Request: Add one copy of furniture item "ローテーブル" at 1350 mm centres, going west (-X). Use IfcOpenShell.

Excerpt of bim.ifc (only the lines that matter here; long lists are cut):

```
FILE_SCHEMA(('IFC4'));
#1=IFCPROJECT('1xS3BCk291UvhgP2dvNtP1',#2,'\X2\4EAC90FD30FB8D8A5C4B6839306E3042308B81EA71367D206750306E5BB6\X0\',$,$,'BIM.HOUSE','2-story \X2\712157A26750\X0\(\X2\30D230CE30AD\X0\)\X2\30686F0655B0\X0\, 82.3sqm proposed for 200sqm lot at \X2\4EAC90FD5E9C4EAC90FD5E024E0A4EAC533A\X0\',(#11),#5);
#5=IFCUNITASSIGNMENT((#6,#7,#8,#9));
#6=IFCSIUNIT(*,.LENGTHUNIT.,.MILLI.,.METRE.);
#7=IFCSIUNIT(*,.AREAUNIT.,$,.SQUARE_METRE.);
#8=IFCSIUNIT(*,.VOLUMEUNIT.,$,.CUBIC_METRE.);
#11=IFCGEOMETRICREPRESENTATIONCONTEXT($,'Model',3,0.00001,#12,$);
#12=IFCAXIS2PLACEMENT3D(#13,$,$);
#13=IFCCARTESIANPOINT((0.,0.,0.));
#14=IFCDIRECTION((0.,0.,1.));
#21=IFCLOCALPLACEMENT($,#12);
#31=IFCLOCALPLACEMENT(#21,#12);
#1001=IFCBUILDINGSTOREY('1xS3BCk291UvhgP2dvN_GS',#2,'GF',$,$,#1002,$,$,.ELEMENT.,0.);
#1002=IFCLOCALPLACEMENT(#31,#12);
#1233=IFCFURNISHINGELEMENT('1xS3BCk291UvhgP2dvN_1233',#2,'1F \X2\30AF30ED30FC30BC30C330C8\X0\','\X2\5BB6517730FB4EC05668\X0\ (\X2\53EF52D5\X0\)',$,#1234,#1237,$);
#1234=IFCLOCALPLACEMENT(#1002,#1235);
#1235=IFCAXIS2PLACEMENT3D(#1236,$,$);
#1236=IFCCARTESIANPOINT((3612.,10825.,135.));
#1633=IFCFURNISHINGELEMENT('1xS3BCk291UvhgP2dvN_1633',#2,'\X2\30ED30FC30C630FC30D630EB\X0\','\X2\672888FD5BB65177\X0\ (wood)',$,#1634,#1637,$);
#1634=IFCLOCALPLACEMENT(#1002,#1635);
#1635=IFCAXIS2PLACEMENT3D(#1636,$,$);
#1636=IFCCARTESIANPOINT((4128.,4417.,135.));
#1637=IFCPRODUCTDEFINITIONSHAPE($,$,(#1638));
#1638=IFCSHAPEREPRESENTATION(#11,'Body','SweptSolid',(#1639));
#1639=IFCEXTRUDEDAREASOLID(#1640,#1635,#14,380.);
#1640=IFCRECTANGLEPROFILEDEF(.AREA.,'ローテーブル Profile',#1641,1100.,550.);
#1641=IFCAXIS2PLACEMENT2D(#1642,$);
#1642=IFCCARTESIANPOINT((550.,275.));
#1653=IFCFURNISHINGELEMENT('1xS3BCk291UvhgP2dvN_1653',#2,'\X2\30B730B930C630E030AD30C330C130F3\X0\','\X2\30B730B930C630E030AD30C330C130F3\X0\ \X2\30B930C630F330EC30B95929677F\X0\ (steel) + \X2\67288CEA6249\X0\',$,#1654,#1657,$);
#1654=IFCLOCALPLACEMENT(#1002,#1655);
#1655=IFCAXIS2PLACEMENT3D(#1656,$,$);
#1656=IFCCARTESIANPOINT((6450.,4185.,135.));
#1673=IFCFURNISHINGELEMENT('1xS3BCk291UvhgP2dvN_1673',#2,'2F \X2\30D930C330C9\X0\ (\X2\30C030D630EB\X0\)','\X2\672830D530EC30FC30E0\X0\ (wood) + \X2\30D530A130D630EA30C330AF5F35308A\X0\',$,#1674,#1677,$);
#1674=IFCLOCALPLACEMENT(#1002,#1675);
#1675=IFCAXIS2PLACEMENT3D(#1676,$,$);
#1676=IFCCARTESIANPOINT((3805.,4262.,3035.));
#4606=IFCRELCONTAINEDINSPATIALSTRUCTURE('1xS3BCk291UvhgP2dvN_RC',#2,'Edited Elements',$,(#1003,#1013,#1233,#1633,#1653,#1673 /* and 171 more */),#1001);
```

```python
import numpy as np
import ifcopenshell
import ifcopenshell.api.geometry
import ifcopenshell.api.root
import ifcopenshell.util.element
import ifcopenshell.util.placement
import ifcopenshell.util.unit

model = ifcopenshell.open("bim.ifc")
unit_scale = ifcopenshell.util.unit.calculate_unit_scale(model)


def reuse_history(source, copy):
    """copy_class also copies each property set's owner history, people and application; keep the originals."""
    for rel in copy.IsDefinedBy:
        if rel.is_a("IfcRelDefinesByProperties") and (history := rel.RelatingPropertyDefinition.OwnerHistory):
            rel.RelatingPropertyDefinition.OwnerHistory = source.OwnerHistory
            ifcopenshell.util.element.remove_deep2(model, history)


source = model.by_guid("1xS3BCk291UvhgP2dvN_1633")
base = ifcopenshell.util.placement.get_local_placement(source.ObjectPlacement)
step = np.array([-1.0, 0.0, 0.0]) * 1.35 / unit_scale

for i in range(1, 2):
    copy = ifcopenshell.api.root.copy_class(model, product=source)
    copy.Representation = ifcopenshell.util.element.copy_deep(
        model, source.Representation, exclude=["IfcGeometricRepresentationContext", "IfcRepresentationMap"]
    )
    reuse_history(source, copy)
    matrix = base.copy()
    matrix[:3, 3] += i * step
    print("added at", matrix[:3, 3].round(3) + 0.0)
    ifcopenshell.api.geometry.edit_object_placement(model, product=copy, matrix=matrix, is_si=False)

model.write("bim_edited.ifc")
```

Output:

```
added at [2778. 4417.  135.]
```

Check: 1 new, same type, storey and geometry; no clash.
